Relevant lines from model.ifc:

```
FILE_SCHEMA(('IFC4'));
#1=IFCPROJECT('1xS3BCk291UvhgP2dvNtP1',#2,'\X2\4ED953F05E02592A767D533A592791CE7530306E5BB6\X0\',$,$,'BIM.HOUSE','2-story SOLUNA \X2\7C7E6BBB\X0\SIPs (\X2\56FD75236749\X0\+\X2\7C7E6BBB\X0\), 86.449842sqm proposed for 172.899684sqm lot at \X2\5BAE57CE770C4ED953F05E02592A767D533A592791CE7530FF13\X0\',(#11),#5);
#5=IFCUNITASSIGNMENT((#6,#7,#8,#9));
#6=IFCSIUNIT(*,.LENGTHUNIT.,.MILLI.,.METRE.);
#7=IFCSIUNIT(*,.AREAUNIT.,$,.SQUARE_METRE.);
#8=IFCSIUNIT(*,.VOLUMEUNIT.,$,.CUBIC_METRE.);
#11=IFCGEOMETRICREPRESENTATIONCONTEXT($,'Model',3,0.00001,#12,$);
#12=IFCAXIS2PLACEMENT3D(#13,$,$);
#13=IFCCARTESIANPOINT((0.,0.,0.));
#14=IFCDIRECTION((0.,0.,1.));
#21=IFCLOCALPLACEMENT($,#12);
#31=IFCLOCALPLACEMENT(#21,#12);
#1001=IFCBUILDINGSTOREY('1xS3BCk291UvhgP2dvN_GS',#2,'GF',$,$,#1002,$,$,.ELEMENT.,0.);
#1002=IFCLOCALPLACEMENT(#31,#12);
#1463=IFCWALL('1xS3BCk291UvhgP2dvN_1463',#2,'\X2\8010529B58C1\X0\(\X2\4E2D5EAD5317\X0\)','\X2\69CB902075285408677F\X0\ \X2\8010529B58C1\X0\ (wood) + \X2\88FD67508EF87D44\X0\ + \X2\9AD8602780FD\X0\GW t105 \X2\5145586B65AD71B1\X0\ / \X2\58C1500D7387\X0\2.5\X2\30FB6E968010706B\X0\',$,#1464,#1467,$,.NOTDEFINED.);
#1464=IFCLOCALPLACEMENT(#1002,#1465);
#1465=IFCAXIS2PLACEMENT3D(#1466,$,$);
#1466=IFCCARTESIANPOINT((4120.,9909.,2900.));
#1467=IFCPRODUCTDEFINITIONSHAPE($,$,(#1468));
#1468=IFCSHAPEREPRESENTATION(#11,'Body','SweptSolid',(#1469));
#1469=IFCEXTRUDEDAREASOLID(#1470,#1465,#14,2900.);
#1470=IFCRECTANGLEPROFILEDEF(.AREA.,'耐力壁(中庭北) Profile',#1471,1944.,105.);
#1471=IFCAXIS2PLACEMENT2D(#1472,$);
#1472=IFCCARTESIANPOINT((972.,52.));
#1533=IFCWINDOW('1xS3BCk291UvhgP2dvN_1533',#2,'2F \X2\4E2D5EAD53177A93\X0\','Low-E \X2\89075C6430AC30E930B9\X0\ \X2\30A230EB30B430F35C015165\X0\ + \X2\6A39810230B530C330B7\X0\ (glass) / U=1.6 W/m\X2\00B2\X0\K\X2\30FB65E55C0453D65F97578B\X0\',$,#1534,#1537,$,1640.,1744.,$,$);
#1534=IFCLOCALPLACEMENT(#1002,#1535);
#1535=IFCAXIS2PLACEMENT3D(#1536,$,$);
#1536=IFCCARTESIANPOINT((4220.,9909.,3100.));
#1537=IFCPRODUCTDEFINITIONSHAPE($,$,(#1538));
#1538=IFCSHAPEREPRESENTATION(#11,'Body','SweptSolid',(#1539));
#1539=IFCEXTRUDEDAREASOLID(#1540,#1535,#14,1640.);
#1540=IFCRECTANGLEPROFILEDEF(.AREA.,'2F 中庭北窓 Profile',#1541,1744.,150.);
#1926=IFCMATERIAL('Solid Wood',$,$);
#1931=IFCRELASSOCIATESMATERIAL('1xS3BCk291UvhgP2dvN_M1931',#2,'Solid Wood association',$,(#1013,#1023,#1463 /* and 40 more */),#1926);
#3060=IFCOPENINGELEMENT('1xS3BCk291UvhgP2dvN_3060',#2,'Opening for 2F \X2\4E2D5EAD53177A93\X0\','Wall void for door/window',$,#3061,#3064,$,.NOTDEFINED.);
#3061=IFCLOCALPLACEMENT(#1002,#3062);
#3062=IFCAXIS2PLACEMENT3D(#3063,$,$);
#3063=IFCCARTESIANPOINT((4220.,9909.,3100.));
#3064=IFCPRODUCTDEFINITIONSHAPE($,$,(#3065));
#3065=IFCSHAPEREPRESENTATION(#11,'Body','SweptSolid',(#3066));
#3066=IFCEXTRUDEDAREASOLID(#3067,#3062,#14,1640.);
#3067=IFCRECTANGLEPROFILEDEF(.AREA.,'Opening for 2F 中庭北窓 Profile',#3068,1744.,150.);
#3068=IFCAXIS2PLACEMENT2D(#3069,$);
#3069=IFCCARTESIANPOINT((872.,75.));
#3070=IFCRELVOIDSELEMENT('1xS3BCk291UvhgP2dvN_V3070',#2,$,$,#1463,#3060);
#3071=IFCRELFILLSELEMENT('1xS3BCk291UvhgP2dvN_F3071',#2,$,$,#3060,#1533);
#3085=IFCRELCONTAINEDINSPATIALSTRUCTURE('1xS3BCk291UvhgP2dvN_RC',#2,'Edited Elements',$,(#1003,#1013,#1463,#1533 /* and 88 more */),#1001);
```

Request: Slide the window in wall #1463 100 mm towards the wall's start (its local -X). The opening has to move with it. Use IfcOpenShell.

```python
import ifcopenshell
import ifcopenshell.api.geometry
import ifcopenshell.util.placement
import ifcopenshell.util.unit

model = ifcopenshell.open("model.ifc")
unit_scale = ifcopenshell.util.unit.calculate_unit_scale(model)

window = model.by_id(1533)
opening = window.FillsVoids[0].RelatingOpeningElement
wall = opening.VoidsElements[0].RelatingBuildingElement

wall_matrix = ifcopenshell.util.placement.get_local_placement(wall.ObjectPlacement)
shift = wall_matrix[:3, 0] * -0.1 / unit_scale
before = ifcopenshell.util.placement.get_local_placement(window.ObjectPlacement)[:3, 3].copy()

# The window is not placed relative to its opening, so move both.
for product in (opening, window):
    matrix = ifcopenshell.util.placement.get_local_placement(product.ObjectPlacement)
    matrix[:3, 3] += shift
    ifcopenshell.api.geometry.edit_object_placement(model, product=product, matrix=matrix, is_si=False)

after = ifcopenshell.util.placement.get_local_placement(window.ObjectPlacement)[:3, 3]
print("window moved by", (after - before).round(3) + 0.0)

model.write("model_rev.ifc")
```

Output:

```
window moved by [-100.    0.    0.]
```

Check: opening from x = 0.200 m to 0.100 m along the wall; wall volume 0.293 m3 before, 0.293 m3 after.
